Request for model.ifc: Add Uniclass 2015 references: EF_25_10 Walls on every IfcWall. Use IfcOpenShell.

First a look at what the model holds.

```python
import ifcopenshell

model = ifcopenshell.open("model.ifc")
print(model.schema)
print("classifications:", [c.Name for c in model.by_type("IfcClassification")])
for ifc_class in ("IfcDoor", "IfcRoof", "IfcStair", "IfcWall", "IfcWindow"):
    print(ifc_class, len(model.by_type(ifc_class)))
```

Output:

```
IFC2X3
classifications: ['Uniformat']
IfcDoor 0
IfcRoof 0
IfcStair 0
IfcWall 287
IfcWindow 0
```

```python
import ifcopenshell
import ifcopenshell.api.classification

model = ifcopenshell.open("model.ifc")

# IFC2X3 requires Source and Edition and has no link from the project to the system.
system = model.create_entity("IfcClassification", Source="NBS", Edition="2015", Name="Uniclass 2015")

codes = {
    "IfcWall": ("EF_25_10", "Walls"),
}
for ifc_class, (code, name) in codes.items():
    products = model.by_type(ifc_class)
    ifcopenshell.api.classification.add_reference(
        model, products=products, classification=system, identification=code, name=name
    )
    print(code, len(products))

model.write("model_v2.ifc")
```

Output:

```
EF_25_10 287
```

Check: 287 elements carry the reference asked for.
